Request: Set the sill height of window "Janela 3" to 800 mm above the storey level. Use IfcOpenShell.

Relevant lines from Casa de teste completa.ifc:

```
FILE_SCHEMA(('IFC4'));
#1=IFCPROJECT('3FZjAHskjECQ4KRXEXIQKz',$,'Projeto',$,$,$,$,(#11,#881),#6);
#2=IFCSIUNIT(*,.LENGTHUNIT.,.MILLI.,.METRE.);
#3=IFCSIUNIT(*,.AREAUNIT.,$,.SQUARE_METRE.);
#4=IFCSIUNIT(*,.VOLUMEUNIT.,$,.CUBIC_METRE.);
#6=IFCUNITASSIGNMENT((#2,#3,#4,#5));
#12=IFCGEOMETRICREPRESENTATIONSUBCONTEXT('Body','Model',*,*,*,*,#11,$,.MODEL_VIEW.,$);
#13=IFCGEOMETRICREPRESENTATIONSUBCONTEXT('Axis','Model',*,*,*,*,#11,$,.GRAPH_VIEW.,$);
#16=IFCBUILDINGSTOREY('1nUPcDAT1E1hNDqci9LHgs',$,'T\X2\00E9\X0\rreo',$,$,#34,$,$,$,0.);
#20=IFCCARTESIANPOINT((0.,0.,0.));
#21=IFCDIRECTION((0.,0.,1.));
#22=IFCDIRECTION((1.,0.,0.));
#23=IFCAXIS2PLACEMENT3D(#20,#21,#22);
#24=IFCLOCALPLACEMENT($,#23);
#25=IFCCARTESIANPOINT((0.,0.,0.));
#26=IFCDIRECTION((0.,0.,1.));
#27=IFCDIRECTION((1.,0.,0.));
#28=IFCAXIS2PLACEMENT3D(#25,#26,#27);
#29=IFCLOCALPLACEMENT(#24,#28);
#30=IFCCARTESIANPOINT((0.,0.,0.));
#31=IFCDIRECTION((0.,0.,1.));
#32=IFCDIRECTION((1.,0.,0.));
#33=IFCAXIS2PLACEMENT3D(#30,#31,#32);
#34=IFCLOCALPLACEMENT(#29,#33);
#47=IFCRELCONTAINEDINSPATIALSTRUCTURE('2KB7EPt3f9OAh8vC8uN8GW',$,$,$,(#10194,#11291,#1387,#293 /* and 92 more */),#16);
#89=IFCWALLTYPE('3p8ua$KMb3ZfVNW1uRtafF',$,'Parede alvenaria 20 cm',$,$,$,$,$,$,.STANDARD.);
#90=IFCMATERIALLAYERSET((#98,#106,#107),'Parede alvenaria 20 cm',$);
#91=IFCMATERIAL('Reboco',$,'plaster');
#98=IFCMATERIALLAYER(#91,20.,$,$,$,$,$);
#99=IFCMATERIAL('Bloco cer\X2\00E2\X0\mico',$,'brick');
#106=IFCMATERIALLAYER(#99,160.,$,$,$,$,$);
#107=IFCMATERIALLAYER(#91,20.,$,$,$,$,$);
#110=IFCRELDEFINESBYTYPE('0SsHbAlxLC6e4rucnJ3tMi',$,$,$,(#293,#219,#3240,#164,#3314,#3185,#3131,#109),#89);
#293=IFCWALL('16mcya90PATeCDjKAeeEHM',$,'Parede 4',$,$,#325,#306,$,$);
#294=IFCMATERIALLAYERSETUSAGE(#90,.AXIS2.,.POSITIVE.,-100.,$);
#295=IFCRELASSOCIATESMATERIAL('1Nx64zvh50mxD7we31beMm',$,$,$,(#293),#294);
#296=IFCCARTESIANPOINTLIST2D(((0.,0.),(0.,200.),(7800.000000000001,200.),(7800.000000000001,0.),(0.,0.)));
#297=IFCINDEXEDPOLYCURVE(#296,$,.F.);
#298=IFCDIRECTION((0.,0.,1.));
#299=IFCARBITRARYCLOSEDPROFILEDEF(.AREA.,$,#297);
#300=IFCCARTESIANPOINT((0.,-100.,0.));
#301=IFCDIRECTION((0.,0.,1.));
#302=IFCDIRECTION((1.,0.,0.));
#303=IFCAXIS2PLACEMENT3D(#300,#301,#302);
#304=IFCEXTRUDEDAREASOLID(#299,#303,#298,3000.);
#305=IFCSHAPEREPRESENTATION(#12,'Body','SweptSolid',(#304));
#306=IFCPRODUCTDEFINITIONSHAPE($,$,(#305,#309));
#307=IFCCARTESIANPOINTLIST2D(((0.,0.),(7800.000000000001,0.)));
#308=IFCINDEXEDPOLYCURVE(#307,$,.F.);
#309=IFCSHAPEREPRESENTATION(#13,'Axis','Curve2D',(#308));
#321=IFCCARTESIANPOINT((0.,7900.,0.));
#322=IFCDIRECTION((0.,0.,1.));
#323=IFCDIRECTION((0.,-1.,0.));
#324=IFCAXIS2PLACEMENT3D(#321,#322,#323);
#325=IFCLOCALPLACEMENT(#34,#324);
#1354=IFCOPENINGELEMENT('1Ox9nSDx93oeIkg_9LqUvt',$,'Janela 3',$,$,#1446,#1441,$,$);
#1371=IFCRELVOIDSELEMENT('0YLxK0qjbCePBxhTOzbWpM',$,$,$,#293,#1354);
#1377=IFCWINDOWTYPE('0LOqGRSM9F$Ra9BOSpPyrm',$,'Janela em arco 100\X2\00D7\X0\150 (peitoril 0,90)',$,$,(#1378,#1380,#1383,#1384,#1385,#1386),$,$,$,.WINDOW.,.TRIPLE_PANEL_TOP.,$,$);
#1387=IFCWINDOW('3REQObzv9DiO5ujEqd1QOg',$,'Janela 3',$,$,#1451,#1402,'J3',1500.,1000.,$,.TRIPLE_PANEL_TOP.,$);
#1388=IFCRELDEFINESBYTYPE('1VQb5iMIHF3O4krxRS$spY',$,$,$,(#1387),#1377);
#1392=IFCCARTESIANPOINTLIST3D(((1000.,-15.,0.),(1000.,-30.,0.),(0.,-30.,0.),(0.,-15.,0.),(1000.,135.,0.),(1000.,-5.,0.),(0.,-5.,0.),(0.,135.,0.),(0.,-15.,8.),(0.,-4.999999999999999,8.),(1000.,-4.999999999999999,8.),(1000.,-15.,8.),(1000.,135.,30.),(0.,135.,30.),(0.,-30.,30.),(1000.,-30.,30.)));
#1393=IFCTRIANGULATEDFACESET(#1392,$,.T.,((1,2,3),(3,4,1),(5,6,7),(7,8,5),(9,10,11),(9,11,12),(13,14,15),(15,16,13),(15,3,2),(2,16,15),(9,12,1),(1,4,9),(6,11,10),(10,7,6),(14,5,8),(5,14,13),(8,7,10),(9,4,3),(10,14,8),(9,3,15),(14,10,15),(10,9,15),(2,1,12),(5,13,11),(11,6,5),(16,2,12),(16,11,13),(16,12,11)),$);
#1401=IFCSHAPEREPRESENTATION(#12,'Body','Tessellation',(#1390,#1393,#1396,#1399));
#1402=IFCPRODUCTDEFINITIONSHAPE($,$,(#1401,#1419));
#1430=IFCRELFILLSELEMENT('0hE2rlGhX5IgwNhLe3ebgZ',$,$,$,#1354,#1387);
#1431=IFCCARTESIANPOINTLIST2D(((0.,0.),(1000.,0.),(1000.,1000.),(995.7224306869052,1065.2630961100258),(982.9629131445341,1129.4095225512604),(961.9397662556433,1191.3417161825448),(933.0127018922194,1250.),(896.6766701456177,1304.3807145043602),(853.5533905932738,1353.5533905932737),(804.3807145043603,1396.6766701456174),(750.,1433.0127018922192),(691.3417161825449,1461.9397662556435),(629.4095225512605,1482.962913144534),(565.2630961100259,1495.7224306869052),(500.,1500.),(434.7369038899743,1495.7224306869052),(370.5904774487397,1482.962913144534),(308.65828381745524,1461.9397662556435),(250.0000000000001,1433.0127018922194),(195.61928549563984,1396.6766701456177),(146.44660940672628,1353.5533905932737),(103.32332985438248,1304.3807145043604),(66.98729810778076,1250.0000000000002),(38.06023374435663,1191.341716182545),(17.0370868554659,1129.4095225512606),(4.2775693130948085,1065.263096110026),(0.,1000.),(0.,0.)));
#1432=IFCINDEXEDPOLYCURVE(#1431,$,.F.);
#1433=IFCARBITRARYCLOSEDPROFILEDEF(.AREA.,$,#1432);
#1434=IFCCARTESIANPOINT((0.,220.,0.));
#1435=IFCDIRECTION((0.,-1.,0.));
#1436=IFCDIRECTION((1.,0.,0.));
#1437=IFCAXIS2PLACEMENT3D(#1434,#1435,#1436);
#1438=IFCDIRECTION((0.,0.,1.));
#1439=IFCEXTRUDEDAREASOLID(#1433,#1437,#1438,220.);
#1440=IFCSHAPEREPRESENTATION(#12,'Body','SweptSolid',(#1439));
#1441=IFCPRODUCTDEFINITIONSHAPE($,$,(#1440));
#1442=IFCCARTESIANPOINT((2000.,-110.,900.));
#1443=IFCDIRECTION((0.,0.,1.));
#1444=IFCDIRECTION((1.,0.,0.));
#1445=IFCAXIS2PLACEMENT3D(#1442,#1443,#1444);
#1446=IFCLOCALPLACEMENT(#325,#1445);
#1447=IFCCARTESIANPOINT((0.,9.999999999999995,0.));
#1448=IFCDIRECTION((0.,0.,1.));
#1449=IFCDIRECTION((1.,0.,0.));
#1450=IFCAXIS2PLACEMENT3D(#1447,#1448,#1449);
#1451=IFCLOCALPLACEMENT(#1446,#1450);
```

```python
import numpy as np
import ifcopenshell
import ifcopenshell.api.geometry
import ifcopenshell.geom
import ifcopenshell.util.element
import ifcopenshell.util.placement
import ifcopenshell.util.shape
import ifcopenshell.util.unit

model = ifcopenshell.open("Casa de teste completa.ifc")
unit_scale = ifcopenshell.util.unit.calculate_unit_scale(model)

window = model.by_guid("3REQObzv9DiO5ujEqd1QOg")
opening = window.FillsVoids[0].RelatingOpeningElement
storey = ifcopenshell.util.element.get_container(window, ifc_class="IfcBuildingStorey")
level = ifcopenshell.util.placement.get_local_placement(storey.ObjectPlacement)[2, 3]

# The opening's origin need not be at the sill, so measure its lowest point.
shape = ifcopenshell.geom.create_shape(ifcopenshell.geom.settings(), opening)
bottom = ifcopenshell.util.shape.get_shape_bottom_elevation(shape, shape.geometry) / unit_scale
dz = level + 0.8 / unit_scale - bottom

shift = np.array([0.0, 0.0, dz])
# The window is placed relative to its opening, so it follows when the opening moves.
matrix = ifcopenshell.util.placement.get_local_placement(opening.ObjectPlacement)
matrix[:3, 3] += shift
ifcopenshell.api.geometry.edit_object_placement(
    model, product=opening, matrix=matrix, is_si=False, should_transform_children=True
)

print(f"moved by {dz * unit_scale:+.3f} m")

model.write("Casa de teste completa_v2.ifc")
```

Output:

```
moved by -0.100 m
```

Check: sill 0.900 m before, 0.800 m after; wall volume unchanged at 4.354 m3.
